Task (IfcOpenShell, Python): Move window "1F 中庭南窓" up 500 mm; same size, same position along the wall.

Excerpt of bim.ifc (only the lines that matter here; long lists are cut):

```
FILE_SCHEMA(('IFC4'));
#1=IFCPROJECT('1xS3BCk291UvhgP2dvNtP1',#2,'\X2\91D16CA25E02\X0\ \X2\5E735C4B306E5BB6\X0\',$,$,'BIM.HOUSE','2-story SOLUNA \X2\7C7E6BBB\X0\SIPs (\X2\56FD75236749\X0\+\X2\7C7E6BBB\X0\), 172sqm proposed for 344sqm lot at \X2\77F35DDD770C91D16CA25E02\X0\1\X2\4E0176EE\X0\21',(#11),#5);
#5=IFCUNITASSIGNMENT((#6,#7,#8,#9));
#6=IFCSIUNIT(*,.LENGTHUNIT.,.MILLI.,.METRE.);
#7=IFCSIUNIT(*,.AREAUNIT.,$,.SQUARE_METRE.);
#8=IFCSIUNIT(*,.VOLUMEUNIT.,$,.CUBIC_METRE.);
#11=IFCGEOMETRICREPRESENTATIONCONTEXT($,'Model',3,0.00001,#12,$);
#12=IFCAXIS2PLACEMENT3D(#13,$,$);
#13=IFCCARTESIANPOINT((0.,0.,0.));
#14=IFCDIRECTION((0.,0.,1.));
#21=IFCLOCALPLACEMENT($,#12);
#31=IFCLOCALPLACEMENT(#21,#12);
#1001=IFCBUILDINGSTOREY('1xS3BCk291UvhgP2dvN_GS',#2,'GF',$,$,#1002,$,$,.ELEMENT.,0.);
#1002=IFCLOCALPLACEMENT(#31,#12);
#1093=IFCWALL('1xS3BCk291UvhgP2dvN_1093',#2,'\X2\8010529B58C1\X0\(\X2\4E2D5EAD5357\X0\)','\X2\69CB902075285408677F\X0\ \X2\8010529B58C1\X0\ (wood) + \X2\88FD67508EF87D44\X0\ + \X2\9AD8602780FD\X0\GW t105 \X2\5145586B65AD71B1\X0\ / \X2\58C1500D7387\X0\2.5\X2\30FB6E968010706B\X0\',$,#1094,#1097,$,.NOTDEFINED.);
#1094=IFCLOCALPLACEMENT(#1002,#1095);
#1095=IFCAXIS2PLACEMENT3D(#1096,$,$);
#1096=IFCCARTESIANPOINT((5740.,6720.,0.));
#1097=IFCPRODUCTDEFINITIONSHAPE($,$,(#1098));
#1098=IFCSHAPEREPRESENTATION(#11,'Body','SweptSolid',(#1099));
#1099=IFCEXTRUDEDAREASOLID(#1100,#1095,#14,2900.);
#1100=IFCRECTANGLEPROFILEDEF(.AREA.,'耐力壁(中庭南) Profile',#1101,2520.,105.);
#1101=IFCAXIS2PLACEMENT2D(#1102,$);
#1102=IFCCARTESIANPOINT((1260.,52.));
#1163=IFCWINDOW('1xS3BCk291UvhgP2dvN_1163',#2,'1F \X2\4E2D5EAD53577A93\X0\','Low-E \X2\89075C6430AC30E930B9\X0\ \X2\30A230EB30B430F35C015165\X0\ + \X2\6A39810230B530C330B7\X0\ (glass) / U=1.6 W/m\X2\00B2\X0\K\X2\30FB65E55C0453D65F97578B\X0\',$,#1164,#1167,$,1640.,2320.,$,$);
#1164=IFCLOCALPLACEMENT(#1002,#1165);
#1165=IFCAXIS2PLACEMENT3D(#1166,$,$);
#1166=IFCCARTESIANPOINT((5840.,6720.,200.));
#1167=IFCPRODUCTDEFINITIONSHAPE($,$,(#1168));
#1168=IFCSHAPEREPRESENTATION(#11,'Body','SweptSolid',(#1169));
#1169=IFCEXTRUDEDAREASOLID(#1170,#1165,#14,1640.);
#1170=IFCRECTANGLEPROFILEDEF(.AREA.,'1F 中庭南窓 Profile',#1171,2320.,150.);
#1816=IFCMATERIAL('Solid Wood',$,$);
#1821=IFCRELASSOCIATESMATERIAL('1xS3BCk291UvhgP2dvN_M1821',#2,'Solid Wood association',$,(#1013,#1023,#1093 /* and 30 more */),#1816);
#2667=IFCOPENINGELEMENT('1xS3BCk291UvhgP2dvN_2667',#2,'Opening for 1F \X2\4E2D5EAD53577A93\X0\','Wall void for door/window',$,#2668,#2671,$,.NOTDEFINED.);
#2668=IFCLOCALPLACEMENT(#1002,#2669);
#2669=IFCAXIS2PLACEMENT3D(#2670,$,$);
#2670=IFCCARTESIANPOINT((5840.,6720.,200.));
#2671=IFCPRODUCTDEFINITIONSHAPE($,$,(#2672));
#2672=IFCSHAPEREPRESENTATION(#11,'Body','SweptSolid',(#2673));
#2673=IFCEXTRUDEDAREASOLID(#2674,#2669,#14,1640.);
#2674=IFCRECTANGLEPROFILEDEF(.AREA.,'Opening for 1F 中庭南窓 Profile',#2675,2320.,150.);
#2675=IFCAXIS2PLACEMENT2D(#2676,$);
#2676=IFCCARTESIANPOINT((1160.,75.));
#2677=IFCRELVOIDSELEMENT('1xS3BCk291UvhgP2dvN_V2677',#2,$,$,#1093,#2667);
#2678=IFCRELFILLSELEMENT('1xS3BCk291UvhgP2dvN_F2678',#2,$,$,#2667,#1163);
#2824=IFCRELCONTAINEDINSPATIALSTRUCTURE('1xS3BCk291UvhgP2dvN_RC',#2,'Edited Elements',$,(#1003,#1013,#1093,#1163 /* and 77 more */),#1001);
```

```python
import numpy as np
import ifcopenshell
import ifcopenshell.api.geometry
import ifcopenshell.util.placement
import ifcopenshell.util.unit

model = ifcopenshell.open("bim.ifc")
unit_scale = ifcopenshell.util.unit.calculate_unit_scale(model)

window = model.by_guid("1xS3BCk291UvhgP2dvN_1163")
opening = window.FillsVoids[0].RelatingOpeningElement
dz = 0.5 / unit_scale

shift = np.array([0.0, 0.0, dz])
# The window is not placed relative to its opening, so move both.
for product in (opening, window):
    matrix = ifcopenshell.util.placement.get_local_placement(product.ObjectPlacement)
    matrix[:3, 3] += shift
    ifcopenshell.api.geometry.edit_object_placement(model, product=product, matrix=matrix, is_si=False)

print(f"moved by {dz * unit_scale:+.3f} m")

model.write("bim-out.ifc")
```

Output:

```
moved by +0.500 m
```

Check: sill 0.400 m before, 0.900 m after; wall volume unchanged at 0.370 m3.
